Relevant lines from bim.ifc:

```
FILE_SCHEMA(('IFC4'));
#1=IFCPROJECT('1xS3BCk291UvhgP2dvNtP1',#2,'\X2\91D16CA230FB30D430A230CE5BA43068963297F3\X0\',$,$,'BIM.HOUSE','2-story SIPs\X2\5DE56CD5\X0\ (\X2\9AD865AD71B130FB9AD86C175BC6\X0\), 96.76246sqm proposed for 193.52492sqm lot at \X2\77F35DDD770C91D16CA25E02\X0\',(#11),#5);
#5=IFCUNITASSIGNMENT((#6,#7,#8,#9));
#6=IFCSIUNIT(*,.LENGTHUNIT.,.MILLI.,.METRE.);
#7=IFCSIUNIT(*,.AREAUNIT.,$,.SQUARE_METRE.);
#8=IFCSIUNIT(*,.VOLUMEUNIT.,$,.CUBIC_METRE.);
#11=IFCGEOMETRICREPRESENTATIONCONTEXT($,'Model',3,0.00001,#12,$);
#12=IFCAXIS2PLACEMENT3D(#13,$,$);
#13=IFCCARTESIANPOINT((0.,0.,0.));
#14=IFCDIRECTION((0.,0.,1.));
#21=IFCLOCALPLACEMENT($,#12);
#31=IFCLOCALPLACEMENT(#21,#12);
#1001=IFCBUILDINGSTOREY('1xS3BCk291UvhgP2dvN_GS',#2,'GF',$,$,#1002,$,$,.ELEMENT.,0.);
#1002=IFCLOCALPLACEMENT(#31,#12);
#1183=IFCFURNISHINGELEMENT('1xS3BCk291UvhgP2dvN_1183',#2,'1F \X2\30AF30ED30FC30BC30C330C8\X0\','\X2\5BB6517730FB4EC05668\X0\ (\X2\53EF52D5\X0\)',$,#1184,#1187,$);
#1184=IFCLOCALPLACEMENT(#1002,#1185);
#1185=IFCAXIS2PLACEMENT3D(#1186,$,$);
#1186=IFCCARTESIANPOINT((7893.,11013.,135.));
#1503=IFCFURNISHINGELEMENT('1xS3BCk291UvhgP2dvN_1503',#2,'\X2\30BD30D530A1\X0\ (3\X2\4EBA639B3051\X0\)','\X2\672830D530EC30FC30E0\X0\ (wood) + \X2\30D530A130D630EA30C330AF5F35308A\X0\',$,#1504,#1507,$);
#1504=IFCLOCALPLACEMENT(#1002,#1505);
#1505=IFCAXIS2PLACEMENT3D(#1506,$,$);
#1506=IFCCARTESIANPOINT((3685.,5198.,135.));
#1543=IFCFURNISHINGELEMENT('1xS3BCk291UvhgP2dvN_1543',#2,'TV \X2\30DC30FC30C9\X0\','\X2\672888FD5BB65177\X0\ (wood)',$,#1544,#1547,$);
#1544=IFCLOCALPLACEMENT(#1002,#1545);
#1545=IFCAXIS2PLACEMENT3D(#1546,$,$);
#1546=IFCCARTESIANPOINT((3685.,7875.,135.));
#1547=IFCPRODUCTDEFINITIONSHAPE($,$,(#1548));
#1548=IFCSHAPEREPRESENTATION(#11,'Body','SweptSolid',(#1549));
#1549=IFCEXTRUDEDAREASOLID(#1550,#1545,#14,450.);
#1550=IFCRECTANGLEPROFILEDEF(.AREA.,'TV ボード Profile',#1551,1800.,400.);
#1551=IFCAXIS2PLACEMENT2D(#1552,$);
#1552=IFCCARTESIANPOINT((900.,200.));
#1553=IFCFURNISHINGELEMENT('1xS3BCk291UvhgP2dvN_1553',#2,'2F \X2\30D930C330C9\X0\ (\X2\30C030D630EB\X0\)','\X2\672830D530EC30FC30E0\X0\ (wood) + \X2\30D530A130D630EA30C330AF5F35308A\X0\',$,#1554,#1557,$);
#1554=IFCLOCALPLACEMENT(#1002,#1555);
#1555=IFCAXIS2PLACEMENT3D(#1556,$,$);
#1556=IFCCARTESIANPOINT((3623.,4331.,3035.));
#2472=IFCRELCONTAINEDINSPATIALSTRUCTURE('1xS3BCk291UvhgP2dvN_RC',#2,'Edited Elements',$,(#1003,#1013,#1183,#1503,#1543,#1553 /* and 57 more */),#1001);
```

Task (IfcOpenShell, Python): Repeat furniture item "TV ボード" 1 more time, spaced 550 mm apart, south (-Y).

```python
import numpy as np
import ifcopenshell
import ifcopenshell.api.geometry
import ifcopenshell.api.root
import ifcopenshell.util.element
import ifcopenshell.util.placement
import ifcopenshell.util.unit

model = ifcopenshell.open("bim.ifc")
unit_scale = ifcopenshell.util.unit.calculate_unit_scale(model)


def reuse_history(source, copy):
    """copy_class also copies each property set's owner history, people and application; keep the originals."""
    for rel in copy.IsDefinedBy:
        if rel.is_a("IfcRelDefinesByProperties") and (history := rel.RelatingPropertyDefinition.OwnerHistory):
            rel.RelatingPropertyDefinition.OwnerHistory = source.OwnerHistory
            ifcopenshell.util.element.remove_deep2(model, history)


source = model.by_guid("1xS3BCk291UvhgP2dvN_1543")
base = ifcopenshell.util.placement.get_local_placement(source.ObjectPlacement)
step = np.array([0.0, -1.0, 0.0]) * 0.55 / unit_scale

for i in range(1, 2):
    copy = ifcopenshell.api.root.copy_class(model, product=source)
    copy.Representation = ifcopenshell.util.element.copy_deep(
        model, source.Representation, exclude=["IfcGeometricRepresentationContext", "IfcRepresentationMap"]
    )
    reuse_history(source, copy)
    matrix = base.copy()
    matrix[:3, 3] += i * step
    print("added at", matrix[:3, 3].round(3) + 0.0)
    ifcopenshell.api.geometry.edit_object_placement(model, product=copy, matrix=matrix, is_si=False)

model.write("bim_updated.ifc")
```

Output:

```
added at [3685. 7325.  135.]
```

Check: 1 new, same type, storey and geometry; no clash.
